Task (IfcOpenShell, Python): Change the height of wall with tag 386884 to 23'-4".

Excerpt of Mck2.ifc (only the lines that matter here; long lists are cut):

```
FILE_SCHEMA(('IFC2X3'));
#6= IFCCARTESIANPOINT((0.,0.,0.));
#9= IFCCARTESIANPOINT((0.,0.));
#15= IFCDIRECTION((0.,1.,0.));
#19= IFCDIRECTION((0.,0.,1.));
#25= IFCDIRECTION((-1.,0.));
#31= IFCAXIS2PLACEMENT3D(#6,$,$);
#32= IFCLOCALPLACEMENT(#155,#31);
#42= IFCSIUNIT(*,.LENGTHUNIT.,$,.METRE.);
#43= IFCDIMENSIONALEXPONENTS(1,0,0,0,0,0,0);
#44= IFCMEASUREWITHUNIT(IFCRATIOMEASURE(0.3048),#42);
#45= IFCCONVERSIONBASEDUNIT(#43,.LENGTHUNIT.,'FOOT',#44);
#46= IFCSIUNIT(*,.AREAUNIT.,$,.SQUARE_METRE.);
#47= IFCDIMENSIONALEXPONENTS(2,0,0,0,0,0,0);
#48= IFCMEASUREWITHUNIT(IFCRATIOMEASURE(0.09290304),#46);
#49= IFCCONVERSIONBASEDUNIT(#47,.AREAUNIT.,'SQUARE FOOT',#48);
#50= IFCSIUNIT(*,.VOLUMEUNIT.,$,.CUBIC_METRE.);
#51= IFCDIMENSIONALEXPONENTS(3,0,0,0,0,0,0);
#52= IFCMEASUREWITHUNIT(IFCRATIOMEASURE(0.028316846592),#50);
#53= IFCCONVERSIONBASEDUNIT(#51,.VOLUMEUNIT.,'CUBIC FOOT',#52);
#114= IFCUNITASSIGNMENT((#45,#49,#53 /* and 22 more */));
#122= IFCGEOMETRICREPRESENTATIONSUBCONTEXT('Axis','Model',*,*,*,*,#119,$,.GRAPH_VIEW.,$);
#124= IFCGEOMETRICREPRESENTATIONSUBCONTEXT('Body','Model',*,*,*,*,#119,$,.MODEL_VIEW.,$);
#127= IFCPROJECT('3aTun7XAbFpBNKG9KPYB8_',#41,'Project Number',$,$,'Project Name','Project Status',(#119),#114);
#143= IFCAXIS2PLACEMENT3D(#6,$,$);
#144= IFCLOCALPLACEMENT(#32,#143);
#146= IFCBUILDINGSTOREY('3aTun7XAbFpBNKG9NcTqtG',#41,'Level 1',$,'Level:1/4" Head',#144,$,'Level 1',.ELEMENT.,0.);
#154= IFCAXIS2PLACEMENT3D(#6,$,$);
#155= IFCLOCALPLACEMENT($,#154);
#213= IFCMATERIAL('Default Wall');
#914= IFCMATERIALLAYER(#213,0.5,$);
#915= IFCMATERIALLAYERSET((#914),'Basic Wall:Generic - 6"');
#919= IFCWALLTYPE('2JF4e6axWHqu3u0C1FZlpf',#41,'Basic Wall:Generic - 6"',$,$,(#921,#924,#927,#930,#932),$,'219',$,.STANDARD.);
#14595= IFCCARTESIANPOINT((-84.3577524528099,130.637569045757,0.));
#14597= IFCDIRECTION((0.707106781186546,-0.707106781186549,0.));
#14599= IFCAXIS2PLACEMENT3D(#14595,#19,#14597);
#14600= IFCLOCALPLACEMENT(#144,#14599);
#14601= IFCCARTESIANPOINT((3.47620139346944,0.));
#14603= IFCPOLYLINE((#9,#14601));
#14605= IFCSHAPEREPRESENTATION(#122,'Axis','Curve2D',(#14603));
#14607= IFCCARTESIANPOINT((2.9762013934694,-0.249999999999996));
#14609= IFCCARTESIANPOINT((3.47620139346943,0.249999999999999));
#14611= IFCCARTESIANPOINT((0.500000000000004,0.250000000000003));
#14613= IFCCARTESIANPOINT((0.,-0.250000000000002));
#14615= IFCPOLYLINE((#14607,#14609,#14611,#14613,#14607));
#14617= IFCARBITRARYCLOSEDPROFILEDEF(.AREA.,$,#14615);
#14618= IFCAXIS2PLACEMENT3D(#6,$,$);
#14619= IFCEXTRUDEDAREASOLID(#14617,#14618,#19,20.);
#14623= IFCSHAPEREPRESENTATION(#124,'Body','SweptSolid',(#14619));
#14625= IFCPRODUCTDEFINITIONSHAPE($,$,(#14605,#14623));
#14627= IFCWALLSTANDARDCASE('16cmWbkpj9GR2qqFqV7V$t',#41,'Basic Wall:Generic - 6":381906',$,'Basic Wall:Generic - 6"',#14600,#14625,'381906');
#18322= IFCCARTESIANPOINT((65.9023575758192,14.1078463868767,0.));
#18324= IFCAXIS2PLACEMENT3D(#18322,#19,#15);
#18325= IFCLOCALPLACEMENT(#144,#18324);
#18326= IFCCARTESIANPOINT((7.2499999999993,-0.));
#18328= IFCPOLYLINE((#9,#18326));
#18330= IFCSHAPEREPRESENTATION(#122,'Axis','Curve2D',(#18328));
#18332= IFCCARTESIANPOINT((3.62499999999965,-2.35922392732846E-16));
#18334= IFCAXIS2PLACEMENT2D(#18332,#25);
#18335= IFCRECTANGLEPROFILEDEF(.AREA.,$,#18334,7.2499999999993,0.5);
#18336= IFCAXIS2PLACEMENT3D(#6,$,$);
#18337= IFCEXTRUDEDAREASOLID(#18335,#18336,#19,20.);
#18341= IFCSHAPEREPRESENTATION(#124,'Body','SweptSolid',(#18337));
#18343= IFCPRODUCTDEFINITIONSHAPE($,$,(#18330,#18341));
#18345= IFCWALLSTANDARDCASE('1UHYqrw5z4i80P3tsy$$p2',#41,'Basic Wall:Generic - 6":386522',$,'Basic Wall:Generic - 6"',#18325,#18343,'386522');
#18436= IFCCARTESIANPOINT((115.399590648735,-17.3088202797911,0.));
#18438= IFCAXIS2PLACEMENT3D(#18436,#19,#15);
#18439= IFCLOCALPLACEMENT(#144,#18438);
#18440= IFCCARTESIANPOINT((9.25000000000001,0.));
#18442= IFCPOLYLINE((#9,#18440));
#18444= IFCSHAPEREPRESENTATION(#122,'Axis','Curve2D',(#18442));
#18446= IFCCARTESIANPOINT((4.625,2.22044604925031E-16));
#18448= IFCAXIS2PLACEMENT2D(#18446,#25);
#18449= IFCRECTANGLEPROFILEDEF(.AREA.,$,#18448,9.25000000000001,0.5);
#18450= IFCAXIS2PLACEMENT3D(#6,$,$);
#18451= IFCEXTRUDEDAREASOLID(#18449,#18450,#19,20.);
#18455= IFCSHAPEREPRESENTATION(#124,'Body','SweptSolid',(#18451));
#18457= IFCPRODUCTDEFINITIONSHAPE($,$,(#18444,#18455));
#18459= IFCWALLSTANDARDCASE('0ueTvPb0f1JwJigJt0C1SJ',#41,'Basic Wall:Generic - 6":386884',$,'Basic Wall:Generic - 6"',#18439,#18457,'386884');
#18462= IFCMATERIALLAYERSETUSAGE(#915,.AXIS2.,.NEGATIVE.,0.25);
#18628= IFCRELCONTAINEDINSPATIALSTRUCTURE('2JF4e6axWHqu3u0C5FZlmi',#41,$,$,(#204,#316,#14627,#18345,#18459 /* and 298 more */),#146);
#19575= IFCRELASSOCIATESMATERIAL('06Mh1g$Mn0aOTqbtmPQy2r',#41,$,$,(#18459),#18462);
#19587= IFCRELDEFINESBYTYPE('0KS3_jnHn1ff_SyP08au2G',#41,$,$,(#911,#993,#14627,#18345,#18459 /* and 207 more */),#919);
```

```python
import ifcopenshell
import ifcopenshell.geom
import ifcopenshell.util.representation
import ifcopenshell.util.shape
import ifcopenshell.util.unit

model = ifcopenshell.open("Mck2.ifc")
unit_scale = ifcopenshell.util.unit.calculate_unit_scale(model)
settings = ifcopenshell.geom.settings()


def volume(element):
    """Net volume in cubic metres, openings subtracted."""
    shape = ifcopenshell.geom.create_shape(settings, element)
    return ifcopenshell.util.shape.get_volume(shape.geometry)


wall = model.by_id(18459)
before = volume(wall)

body = ifcopenshell.util.representation.get_representation(wall, "Model", "Body")
solid = body.Items[0]
old_height = solid.Depth
solid.Depth = 280 * 0.0254 / unit_scale
after = volume(wall)

print(f"height {old_height:g} -> {solid.Depth:g}, volume {before:.3f} -> {after:.3f} m3")

model.write("Mck2-out.ifc")
```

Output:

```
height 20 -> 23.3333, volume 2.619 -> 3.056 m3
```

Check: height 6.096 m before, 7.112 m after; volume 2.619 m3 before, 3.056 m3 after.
